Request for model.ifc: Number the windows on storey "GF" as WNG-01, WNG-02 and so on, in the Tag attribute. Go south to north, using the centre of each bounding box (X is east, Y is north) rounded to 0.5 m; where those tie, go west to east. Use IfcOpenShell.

First a look at what the model holds.

```python
import ifcopenshell
import ifcopenshell.util.element
import ifcopenshell.util.placement

model = ifcopenshell.open("model.ifc")
print(model.schema)
storey = next(s for s in model.by_type("IfcBuildingStorey") if s.Name == "GF")
windows = [e for e in ifcopenshell.util.element.get_decomposition(storey) if e.is_a("IfcWindow")]
for e in sorted(windows, key=lambda e: e.id()):
    origin = ifcopenshell.util.placement.get_local_placement(e.ObjectPlacement)[:3, 3]
    print(e.id(), e.Tag, e.Name, origin.round(2) + 0.0, sep=" | ")
```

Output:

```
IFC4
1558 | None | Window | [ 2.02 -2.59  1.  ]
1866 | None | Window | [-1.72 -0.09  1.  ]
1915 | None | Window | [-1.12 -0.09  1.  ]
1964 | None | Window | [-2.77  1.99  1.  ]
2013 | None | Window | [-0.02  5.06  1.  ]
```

```python
import ifcopenshell
import ifcopenshell.geom
import ifcopenshell.util.element
import ifcopenshell.util.shape

model = ifcopenshell.open("model.ifc")
settings = ifcopenshell.geom.settings()
settings.set("use-world-coords", True)


def centre(element):
    shape = ifcopenshell.geom.create_shape(settings, element)
    return ifcopenshell.util.shape.get_bbox_centroid(shape.geometry)


storey = next(s for s in model.by_type("IfcBuildingStorey") if s.Name == "GF")
windows = [e for e in ifcopenshell.util.element.get_decomposition(storey) if e.is_a("IfcWindow")]

# Insertion points can sit at a corner or the storey origin, so sort by the geometry (in metres).
centres = {e: centre(e) for e in windows}
windows.sort(key=lambda e: (round(centres[e][1] / 0.5), centres[e][0]))

for i, e in enumerate(windows, start=1):
    number = f"WNG-{i:02d}"
    e.Tag = number
    print(e.id(), number)

model.write("model_edited.ifc")
```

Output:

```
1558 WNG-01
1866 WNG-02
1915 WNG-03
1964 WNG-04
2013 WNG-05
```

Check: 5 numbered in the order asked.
